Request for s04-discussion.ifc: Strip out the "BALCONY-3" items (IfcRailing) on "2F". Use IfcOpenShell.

First a look at what the model holds.

```python
import ifcopenshell
import ifcopenshell.util.element

model = ifcopenshell.open("s04-discussion.ifc")
print(model.schema)
storey = next(s for s in model.by_type("IfcBuildingStorey") if s.Name == "2F")
railings = [e for e in ifcopenshell.util.element.get_decomposition(storey) if e.is_a("IfcRailing")]
seen = {}
for e in railings:
    element_type = ifcopenshell.util.element.get_type(e)
    name = element_type.Name if element_type not in (None, e) else None
    seen[name] = seen.get(name, 0) + 1
for name, count in sorted(seen.items(), key=str):
    print(count, "x", name)
```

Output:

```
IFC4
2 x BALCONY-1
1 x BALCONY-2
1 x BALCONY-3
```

```python
import ifcopenshell
import ifcopenshell.api.root
import ifcopenshell.util.element

model = ifcopenshell.open("s04-discussion.ifc")

storey = next(s for s in model.by_type("IfcBuildingStorey") if s.Name == "2F")
railings = [e for e in ifcopenshell.util.element.get_decomposition(storey) if e.is_a("IfcRailing")]
targets = [e for e in railings if (t := ifcopenshell.util.element.get_type(e)) not in (None, e) and t.Name == "BALCONY-3"]

for e in targets:
    ifcopenshell.api.root.remove_product(model, product=e)
print(len(targets), "removed")

model.write("s04-discussion_edited.ifc")
```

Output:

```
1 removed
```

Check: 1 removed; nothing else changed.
